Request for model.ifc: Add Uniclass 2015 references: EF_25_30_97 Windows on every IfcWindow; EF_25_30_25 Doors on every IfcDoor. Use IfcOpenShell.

First a look at what the model holds.

```python
import ifcopenshell

model = ifcopenshell.open("model.ifc")
print(model.schema)
print("classifications:", [c.Name for c in model.by_type("IfcClassification")])
for ifc_class in ("IfcDoor", "IfcRoof", "IfcStair", "IfcWall", "IfcWindow"):
    print(ifc_class, len(model.by_type(ifc_class)))
```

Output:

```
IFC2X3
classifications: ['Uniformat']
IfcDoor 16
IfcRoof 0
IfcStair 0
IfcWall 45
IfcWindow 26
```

```python
import ifcopenshell
import ifcopenshell.api.classification

model = ifcopenshell.open("model.ifc")

# IFC2X3 requires Source and Edition and has no link from the project to the system.
system = model.create_entity("IfcClassification", Source="NBS", Edition="2015", Name="Uniclass 2015")

codes = {
    "IfcWindow": ("EF_25_30_97", "Windows"),
    "IfcDoor": ("EF_25_30_25", "Doors"),
}
for ifc_class, (code, name) in codes.items():
    products = model.by_type(ifc_class)
    ifcopenshell.api.classification.add_reference(
        model, products=products, classification=system, identification=code, name=name
    )
    print(code, len(products))

model.write("model-out.ifc")
```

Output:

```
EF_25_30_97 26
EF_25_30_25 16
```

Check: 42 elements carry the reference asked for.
